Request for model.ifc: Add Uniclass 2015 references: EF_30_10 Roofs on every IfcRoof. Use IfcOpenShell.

First a look at what the model holds.

```python
import ifcopenshell

model = ifcopenshell.open("model.ifc")
print(model.schema)
print("classifications:", [c.Name for c in model.by_type("IfcClassification")])
for ifc_class in ("IfcDoor", "IfcRoof", "IfcStair", "IfcWall", "IfcWindow"):
    print(ifc_class, len(model.by_type(ifc_class)))
```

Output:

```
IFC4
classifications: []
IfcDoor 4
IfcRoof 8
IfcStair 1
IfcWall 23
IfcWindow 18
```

```python
import ifcopenshell
import ifcopenshell.api.classification

model = ifcopenshell.open("model.ifc")

system = ifcopenshell.api.classification.add_classification(model, classification="Uniclass 2015")

codes = {
    "IfcRoof": ("EF_30_10", "Roofs"),
}
for ifc_class, (code, name) in codes.items():
    products = model.by_type(ifc_class)
    ifcopenshell.api.classification.add_reference(
        model, products=products, classification=system, identification=code, name=name
    )
    print(code, len(products))

model.write("model_v2.ifc")
```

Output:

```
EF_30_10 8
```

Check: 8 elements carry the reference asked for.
